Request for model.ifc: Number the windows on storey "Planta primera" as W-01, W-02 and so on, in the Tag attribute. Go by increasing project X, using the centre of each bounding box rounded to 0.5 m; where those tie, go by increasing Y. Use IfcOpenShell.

First a look at what the model holds.

```python
import ifcopenshell
import ifcopenshell.util.element
import ifcopenshell.util.placement

model = ifcopenshell.open("model.ifc")
print(model.schema)
storey = next(s for s in model.by_type("IfcBuildingStorey") if s.Name == "Planta primera")
windows = [e for e in ifcopenshell.util.element.get_decomposition(storey) if e.is_a("IfcWindow")]
for e in sorted(windows, key=lambda e: e.id()):
    origin = ifcopenshell.util.placement.get_local_placement(e.ObjectPlacement)[:3, 3]
    print(e.id(), e.Tag, e.Name, origin.round(2) + 0.0, sep=" | ")
```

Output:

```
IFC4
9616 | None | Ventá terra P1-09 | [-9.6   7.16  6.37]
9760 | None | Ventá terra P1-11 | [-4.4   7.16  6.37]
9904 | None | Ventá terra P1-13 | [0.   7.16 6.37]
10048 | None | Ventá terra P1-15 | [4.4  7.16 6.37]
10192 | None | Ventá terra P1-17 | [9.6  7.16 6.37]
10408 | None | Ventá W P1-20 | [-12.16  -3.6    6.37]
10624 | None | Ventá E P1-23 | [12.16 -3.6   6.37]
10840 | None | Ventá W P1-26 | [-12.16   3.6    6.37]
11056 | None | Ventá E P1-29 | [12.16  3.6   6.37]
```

```python
import ifcopenshell
import ifcopenshell.geom
import ifcopenshell.util.element
import ifcopenshell.util.shape

model = ifcopenshell.open("model.ifc")
settings = ifcopenshell.geom.settings()
settings.set("use-world-coords", True)


def centre(element):
    shape = ifcopenshell.geom.create_shape(settings, element)
    return ifcopenshell.util.shape.get_bbox_centroid(shape.geometry)


storey = next(s for s in model.by_type("IfcBuildingStorey") if s.Name == "Planta primera")
windows = [e for e in ifcopenshell.util.element.get_decomposition(storey) if e.is_a("IfcWindow")]

# Insertion points can sit at a corner or the storey origin, so sort by the geometry (in metres).
centres = {e: centre(e) for e in windows}
windows.sort(key=lambda e: (round(centres[e][0] / 0.5), centres[e][1]))

for i, e in enumerate(windows, start=1):
    number = f"W-{i:02d}"
    e.Tag = number
    print(e.id(), number)

model.write("model-out.ifc")
```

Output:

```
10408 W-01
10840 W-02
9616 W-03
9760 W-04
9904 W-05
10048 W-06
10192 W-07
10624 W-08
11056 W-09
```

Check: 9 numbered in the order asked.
